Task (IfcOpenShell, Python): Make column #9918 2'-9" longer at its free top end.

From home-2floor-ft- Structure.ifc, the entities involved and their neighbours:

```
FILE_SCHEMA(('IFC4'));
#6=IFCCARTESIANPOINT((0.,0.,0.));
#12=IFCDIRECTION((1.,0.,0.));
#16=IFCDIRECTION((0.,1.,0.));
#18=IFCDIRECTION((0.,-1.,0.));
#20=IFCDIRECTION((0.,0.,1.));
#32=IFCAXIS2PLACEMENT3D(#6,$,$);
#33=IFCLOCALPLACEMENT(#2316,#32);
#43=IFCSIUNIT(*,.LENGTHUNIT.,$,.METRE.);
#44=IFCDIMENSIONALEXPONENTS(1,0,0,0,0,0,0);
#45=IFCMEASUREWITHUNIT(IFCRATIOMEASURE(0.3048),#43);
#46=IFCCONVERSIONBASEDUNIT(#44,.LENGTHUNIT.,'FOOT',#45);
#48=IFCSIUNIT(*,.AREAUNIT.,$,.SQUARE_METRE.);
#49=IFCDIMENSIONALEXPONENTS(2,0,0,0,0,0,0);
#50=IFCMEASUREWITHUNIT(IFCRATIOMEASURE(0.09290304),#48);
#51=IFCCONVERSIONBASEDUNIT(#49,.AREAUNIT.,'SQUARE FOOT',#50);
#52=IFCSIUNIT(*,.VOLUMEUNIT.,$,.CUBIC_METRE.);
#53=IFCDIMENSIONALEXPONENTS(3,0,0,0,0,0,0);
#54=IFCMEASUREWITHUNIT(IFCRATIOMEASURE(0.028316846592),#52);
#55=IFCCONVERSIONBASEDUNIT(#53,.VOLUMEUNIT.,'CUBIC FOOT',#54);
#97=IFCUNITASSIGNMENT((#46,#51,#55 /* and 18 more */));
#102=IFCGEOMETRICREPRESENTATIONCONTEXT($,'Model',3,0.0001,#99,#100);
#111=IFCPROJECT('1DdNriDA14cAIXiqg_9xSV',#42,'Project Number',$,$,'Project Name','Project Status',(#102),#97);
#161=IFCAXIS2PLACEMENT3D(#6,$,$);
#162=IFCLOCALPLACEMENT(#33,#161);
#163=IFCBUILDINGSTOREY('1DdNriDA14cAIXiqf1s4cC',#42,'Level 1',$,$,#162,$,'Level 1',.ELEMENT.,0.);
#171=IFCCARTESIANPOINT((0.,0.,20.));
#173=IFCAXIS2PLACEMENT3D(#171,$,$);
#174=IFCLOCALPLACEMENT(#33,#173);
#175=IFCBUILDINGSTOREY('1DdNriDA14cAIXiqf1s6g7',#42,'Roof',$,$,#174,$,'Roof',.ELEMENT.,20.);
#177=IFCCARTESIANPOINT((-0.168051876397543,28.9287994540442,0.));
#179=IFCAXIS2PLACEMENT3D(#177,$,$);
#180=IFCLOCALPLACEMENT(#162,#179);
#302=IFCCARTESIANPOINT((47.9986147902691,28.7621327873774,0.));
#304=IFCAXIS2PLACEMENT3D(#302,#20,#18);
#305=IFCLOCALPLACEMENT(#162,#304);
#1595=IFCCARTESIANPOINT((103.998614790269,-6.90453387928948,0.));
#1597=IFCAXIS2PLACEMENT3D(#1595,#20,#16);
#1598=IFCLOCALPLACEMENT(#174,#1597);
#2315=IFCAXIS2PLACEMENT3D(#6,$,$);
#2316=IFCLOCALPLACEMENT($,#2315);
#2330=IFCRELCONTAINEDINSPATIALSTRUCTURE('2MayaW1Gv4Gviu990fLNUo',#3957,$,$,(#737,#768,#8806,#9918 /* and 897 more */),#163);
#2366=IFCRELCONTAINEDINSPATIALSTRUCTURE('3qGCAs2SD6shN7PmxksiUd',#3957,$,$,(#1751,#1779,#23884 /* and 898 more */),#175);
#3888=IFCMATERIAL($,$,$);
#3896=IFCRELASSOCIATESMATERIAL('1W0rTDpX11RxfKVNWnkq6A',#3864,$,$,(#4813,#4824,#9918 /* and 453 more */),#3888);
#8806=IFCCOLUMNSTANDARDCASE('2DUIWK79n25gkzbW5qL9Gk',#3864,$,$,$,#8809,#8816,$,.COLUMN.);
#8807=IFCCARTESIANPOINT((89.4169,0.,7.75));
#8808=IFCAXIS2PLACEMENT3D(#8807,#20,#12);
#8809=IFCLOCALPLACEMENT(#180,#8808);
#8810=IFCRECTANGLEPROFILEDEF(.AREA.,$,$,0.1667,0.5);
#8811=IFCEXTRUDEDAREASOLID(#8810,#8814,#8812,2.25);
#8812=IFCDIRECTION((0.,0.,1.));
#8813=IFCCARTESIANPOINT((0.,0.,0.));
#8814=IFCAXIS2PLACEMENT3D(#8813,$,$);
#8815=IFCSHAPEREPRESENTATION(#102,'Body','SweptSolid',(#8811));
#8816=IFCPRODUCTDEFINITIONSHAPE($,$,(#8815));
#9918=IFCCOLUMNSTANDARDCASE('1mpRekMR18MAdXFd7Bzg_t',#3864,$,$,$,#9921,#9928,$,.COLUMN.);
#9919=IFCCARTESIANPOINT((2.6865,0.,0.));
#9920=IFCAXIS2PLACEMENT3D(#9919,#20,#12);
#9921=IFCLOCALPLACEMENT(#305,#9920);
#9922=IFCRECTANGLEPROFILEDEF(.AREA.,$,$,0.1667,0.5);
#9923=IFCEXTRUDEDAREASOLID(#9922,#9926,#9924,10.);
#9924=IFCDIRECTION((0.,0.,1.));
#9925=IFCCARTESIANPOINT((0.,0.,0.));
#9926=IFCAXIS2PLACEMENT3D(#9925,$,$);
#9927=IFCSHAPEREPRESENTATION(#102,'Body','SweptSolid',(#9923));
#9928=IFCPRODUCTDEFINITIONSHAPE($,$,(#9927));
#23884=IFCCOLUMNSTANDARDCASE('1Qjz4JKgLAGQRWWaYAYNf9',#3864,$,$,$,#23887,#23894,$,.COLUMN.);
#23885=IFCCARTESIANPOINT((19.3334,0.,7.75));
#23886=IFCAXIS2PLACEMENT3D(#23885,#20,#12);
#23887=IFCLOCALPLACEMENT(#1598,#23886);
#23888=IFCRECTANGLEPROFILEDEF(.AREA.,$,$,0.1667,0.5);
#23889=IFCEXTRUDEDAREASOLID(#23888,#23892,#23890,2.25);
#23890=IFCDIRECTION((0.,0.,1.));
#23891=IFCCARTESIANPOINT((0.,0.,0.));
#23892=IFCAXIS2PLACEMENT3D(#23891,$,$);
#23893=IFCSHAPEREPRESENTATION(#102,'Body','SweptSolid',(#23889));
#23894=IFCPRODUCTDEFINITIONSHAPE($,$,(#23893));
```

```python
import ifcopenshell
import ifcopenshell.util.unit

model = ifcopenshell.open("home-2floor-ft- Structure.ifc")
unit_scale = ifcopenshell.util.unit.calculate_unit_scale(model)

member = model.by_id(9918)
change = 33 * 0.0254 / unit_scale

# The extrusion runs towards the end named, so only its depth changes.
body = next(r for r in member.Representation.Representations if r.RepresentationIdentifier == "Body")
solid = body.Items[0]
old_length = solid.Depth
solid.Depth += change

print(f"length {old_length:g} -> {solid.Depth:g}")

model.write("home-2floor-ft- Structure_edited.ifc")
```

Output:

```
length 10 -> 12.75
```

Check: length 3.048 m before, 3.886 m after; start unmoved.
